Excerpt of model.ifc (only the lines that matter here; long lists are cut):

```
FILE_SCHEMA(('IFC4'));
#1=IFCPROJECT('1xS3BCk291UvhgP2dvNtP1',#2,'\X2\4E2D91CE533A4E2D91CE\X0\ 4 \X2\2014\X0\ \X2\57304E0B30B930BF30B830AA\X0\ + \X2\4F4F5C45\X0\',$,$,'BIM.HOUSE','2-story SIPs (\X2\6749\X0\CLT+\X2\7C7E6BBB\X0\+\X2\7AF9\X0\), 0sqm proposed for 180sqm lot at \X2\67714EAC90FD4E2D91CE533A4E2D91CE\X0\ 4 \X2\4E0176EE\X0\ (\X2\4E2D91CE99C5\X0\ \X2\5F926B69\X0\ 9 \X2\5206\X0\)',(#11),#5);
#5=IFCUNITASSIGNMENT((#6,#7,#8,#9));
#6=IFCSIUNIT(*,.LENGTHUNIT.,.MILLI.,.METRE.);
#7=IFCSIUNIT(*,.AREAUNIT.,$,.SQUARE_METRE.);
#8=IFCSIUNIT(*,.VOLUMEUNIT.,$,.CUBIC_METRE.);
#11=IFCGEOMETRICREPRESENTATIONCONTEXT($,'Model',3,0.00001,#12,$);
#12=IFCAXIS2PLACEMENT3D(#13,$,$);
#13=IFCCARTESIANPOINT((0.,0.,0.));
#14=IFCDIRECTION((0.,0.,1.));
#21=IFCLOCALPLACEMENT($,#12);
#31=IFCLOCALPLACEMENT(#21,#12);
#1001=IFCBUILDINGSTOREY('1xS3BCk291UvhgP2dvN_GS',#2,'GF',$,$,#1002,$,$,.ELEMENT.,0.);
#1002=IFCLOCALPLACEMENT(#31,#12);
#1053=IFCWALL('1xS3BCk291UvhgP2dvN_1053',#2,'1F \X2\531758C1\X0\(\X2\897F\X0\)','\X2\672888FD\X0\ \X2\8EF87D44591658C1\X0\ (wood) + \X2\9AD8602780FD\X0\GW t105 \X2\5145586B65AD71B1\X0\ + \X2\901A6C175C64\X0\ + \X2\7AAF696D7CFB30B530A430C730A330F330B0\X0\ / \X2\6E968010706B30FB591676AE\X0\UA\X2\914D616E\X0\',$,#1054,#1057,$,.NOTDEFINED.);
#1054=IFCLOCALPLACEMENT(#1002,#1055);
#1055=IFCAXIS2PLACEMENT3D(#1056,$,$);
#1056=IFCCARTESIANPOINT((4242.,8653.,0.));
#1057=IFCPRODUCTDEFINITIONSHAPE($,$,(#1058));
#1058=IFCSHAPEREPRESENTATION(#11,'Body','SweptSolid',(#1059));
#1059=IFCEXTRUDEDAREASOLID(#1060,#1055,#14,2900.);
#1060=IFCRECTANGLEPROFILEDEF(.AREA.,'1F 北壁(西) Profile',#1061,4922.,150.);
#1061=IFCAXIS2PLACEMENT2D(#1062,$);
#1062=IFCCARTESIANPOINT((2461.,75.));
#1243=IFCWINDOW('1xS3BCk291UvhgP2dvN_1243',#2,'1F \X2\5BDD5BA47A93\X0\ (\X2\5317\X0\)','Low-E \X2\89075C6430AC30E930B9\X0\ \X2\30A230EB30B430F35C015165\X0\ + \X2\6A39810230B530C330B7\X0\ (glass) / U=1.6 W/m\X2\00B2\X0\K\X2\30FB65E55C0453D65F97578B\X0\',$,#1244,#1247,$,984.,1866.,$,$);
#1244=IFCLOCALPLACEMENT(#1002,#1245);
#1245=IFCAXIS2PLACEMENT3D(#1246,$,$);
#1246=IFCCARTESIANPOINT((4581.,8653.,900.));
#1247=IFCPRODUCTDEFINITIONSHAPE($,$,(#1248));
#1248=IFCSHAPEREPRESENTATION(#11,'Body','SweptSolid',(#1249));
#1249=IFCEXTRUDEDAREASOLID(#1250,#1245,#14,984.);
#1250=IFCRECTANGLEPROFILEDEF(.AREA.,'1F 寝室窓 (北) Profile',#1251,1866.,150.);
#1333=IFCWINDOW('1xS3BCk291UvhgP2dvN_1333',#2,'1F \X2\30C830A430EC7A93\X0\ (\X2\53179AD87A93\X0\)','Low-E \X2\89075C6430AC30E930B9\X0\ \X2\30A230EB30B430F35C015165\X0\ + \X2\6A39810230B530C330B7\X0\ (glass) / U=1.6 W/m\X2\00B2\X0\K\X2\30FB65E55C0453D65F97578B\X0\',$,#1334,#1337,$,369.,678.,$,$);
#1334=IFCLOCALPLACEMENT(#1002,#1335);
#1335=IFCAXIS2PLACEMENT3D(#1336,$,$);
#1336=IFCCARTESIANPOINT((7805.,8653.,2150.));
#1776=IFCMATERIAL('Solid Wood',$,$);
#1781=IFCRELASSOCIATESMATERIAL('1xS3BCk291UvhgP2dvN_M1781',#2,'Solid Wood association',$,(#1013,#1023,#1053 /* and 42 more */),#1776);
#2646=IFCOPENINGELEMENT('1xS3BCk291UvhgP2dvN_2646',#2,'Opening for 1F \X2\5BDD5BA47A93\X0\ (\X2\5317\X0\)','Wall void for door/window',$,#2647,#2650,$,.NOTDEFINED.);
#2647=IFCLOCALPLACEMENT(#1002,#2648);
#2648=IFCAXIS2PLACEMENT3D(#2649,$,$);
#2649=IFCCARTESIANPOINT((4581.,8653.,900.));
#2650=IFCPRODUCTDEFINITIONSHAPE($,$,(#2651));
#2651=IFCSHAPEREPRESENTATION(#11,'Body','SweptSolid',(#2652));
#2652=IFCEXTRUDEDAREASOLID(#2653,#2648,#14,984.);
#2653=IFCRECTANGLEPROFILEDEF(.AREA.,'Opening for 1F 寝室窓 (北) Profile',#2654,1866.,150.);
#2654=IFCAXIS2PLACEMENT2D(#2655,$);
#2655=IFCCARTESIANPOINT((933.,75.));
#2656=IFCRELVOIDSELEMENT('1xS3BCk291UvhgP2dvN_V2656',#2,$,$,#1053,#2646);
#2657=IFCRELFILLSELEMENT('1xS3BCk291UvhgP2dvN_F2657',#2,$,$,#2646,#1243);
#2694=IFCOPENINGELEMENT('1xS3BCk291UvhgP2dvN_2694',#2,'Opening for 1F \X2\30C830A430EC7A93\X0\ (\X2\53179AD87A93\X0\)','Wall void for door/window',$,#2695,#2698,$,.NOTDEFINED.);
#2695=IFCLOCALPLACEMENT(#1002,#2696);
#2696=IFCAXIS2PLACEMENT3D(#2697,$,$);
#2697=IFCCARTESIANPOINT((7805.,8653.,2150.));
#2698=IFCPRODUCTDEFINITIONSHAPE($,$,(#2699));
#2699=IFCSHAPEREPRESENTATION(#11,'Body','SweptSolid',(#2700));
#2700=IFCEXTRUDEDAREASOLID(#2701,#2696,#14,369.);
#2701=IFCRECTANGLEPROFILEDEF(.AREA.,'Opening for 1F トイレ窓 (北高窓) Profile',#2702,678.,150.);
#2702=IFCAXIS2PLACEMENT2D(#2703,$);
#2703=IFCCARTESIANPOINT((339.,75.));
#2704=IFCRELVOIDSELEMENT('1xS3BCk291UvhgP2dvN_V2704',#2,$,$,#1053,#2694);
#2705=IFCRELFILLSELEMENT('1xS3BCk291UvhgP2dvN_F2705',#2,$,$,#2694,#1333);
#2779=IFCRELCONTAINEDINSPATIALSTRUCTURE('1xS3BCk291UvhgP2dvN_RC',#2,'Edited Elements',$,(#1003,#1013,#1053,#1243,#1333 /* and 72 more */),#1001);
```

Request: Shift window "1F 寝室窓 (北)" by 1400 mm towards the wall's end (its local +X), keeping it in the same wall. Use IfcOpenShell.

```python
import ifcopenshell
import ifcopenshell.api.geometry
import ifcopenshell.util.placement
import ifcopenshell.util.unit

model = ifcopenshell.open("model.ifc")
unit_scale = ifcopenshell.util.unit.calculate_unit_scale(model)

window = model.by_guid("1xS3BCk291UvhgP2dvN_1243")
opening = window.FillsVoids[0].RelatingOpeningElement
wall = opening.VoidsElements[0].RelatingBuildingElement

wall_matrix = ifcopenshell.util.placement.get_local_placement(wall.ObjectPlacement)
shift = wall_matrix[:3, 0] * 1.4 / unit_scale
before = ifcopenshell.util.placement.get_local_placement(window.ObjectPlacement)[:3, 3].copy()

# The window is not placed relative to its opening, so move both.
for product in (opening, window):
    matrix = ifcopenshell.util.placement.get_local_placement(product.ObjectPlacement)
    matrix[:3, 3] += shift
    ifcopenshell.api.geometry.edit_object_placement(model, product=product, matrix=matrix, is_si=False)

after = ifcopenshell.util.placement.get_local_placement(window.ObjectPlacement)[:3, 3]
print("window moved by", (after - before).round(3) + 0.0)

model.write("model_edited.ifc")
```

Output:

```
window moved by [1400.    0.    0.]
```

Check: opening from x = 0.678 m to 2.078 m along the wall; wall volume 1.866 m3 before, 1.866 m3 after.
